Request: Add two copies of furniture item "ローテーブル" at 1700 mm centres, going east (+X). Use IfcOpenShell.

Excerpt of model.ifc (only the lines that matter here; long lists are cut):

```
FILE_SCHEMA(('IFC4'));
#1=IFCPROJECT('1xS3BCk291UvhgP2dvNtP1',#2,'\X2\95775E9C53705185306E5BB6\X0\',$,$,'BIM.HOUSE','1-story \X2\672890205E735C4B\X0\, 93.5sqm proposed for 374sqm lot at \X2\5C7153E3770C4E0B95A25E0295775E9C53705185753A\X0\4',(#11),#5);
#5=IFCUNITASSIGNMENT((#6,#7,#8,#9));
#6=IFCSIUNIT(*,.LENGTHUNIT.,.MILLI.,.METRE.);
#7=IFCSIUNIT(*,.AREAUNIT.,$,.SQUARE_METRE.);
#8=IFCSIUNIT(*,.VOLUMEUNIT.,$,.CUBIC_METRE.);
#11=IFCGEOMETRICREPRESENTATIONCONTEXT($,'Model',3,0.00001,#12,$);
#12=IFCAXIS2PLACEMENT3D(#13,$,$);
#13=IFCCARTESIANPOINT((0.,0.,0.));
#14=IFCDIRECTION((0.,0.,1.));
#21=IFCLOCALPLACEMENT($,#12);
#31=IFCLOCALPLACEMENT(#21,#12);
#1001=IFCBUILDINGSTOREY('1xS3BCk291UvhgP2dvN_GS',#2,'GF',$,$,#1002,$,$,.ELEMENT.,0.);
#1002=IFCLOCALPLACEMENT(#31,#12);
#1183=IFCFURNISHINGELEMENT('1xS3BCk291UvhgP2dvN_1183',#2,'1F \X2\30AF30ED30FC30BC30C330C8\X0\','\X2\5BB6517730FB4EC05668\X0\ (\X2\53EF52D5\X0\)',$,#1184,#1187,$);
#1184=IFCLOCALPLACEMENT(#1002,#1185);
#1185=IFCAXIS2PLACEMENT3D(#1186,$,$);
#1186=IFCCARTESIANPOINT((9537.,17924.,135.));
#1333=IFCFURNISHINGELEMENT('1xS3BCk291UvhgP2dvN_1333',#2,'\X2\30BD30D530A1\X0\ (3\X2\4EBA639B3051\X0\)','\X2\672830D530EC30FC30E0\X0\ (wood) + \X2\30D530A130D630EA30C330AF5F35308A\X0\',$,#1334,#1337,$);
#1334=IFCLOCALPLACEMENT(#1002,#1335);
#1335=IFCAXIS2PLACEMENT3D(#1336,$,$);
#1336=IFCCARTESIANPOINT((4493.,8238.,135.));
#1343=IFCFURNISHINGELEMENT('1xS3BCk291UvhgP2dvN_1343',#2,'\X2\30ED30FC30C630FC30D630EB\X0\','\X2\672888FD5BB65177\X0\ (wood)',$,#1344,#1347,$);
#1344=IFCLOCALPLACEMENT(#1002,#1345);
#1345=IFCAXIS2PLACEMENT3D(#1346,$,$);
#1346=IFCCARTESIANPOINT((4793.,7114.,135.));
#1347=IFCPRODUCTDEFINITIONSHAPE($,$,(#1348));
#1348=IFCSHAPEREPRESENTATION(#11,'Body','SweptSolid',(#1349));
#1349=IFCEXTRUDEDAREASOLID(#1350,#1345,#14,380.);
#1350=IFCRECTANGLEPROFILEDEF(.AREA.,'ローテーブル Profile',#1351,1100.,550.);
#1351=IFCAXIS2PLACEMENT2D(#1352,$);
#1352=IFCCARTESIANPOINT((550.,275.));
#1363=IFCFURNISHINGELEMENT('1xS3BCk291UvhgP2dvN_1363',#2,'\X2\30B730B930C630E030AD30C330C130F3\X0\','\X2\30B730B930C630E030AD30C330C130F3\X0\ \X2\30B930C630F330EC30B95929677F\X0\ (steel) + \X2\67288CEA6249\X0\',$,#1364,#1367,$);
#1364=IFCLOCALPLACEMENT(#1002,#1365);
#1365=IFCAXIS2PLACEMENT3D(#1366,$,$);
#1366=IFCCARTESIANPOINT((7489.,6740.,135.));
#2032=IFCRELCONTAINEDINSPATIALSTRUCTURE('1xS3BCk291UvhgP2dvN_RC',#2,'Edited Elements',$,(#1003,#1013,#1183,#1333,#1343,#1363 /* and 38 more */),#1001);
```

```python
import numpy as np
import ifcopenshell
import ifcopenshell.api.geometry
import ifcopenshell.api.root
import ifcopenshell.util.element
import ifcopenshell.util.placement

model = ifcopenshell.open("model.ifc")


def reuse_history(source, copy):
    """copy_class also copies each property set's owner history, people and application; keep the originals."""
    for rel in copy.IsDefinedBy:
        if rel.is_a("IfcRelDefinesByProperties") and (history := rel.RelatingPropertyDefinition.OwnerHistory):
            rel.RelatingPropertyDefinition.OwnerHistory = source.OwnerHistory
            ifcopenshell.util.element.remove_deep2(model, history)


source = model.by_guid("1xS3BCk291UvhgP2dvN_1343")
base = ifcopenshell.util.placement.get_local_placement(source.ObjectPlacement)
step = np.array([1.0, 0.0, 0.0]) * 1700.0

for i in range(1, 3):
    copy = ifcopenshell.api.root.copy_class(model, product=source)
    copy.Representation = ifcopenshell.util.element.copy_deep(
        model, source.Representation, exclude=["IfcGeometricRepresentationContext", "IfcRepresentationMap"]
    )
    reuse_history(source, copy)
    matrix = base.copy()
    matrix[:3, 3] += i * step
    print("added at", matrix[:3, 3].round(3) + 0.0)
    ifcopenshell.api.geometry.edit_object_placement(model, product=copy, matrix=matrix, is_si=False)

model.write("model_edited.ifc")
```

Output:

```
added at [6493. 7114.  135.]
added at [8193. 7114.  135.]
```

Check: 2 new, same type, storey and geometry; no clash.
